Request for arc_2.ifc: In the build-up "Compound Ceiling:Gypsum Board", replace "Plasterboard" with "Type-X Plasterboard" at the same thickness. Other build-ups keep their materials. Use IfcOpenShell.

First a look at what the model holds.

```python
import ifcopenshell
import ifcopenshell.util.element

model = ifcopenshell.open("arc_2.ifc")
print(model.schema)
for layer_set in model.by_type("IfcMaterialLayerSet"):
    if layer_set.LayerSetName == "Compound Ceiling:Gypsum Board":
        for layer in layer_set.MaterialLayers:
            print(layer.id(), layer.Material and layer.Material.Name, layer.LayerThickness, sep=" | ")
        print(len(ifcopenshell.util.element.get_elements_by_material(model, layer_set)), "elements and types use it")
print(sorted(m.Name for m in model.by_type("IfcMaterial") if m.Name)[:60])
```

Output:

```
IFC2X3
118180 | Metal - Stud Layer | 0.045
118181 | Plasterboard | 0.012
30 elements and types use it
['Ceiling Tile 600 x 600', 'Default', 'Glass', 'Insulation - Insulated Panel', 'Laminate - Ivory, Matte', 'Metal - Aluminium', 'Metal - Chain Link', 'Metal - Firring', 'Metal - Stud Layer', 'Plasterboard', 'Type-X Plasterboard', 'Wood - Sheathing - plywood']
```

```python
import ifcopenshell
import ifcopenshell.api.material

model = ifcopenshell.open("arc_2.ifc")

layer_set = next(s for s in model.by_type("IfcMaterialLayerSet") if s.LayerSetName == "Compound Ceiling:Gypsum Board")
layer = next(l for l in layer_set.MaterialLayers if l.Material and l.Material.Name == "Plasterboard")
material = next(m for m in model.by_type("IfcMaterial") if m.Name == "Type-X Plasterboard")

# Point this one layer at the other material; renaming the old one would change it everywhere.
ifcopenshell.api.material.edit_layer(model, layer=layer, attributes={}, material=material)

print([l.Material.Name if l.Material else None for l in layer_set.MaterialLayers])

model.write("arc_2_rev.ifc")
```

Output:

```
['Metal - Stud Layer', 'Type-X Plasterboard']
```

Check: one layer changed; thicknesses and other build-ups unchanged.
